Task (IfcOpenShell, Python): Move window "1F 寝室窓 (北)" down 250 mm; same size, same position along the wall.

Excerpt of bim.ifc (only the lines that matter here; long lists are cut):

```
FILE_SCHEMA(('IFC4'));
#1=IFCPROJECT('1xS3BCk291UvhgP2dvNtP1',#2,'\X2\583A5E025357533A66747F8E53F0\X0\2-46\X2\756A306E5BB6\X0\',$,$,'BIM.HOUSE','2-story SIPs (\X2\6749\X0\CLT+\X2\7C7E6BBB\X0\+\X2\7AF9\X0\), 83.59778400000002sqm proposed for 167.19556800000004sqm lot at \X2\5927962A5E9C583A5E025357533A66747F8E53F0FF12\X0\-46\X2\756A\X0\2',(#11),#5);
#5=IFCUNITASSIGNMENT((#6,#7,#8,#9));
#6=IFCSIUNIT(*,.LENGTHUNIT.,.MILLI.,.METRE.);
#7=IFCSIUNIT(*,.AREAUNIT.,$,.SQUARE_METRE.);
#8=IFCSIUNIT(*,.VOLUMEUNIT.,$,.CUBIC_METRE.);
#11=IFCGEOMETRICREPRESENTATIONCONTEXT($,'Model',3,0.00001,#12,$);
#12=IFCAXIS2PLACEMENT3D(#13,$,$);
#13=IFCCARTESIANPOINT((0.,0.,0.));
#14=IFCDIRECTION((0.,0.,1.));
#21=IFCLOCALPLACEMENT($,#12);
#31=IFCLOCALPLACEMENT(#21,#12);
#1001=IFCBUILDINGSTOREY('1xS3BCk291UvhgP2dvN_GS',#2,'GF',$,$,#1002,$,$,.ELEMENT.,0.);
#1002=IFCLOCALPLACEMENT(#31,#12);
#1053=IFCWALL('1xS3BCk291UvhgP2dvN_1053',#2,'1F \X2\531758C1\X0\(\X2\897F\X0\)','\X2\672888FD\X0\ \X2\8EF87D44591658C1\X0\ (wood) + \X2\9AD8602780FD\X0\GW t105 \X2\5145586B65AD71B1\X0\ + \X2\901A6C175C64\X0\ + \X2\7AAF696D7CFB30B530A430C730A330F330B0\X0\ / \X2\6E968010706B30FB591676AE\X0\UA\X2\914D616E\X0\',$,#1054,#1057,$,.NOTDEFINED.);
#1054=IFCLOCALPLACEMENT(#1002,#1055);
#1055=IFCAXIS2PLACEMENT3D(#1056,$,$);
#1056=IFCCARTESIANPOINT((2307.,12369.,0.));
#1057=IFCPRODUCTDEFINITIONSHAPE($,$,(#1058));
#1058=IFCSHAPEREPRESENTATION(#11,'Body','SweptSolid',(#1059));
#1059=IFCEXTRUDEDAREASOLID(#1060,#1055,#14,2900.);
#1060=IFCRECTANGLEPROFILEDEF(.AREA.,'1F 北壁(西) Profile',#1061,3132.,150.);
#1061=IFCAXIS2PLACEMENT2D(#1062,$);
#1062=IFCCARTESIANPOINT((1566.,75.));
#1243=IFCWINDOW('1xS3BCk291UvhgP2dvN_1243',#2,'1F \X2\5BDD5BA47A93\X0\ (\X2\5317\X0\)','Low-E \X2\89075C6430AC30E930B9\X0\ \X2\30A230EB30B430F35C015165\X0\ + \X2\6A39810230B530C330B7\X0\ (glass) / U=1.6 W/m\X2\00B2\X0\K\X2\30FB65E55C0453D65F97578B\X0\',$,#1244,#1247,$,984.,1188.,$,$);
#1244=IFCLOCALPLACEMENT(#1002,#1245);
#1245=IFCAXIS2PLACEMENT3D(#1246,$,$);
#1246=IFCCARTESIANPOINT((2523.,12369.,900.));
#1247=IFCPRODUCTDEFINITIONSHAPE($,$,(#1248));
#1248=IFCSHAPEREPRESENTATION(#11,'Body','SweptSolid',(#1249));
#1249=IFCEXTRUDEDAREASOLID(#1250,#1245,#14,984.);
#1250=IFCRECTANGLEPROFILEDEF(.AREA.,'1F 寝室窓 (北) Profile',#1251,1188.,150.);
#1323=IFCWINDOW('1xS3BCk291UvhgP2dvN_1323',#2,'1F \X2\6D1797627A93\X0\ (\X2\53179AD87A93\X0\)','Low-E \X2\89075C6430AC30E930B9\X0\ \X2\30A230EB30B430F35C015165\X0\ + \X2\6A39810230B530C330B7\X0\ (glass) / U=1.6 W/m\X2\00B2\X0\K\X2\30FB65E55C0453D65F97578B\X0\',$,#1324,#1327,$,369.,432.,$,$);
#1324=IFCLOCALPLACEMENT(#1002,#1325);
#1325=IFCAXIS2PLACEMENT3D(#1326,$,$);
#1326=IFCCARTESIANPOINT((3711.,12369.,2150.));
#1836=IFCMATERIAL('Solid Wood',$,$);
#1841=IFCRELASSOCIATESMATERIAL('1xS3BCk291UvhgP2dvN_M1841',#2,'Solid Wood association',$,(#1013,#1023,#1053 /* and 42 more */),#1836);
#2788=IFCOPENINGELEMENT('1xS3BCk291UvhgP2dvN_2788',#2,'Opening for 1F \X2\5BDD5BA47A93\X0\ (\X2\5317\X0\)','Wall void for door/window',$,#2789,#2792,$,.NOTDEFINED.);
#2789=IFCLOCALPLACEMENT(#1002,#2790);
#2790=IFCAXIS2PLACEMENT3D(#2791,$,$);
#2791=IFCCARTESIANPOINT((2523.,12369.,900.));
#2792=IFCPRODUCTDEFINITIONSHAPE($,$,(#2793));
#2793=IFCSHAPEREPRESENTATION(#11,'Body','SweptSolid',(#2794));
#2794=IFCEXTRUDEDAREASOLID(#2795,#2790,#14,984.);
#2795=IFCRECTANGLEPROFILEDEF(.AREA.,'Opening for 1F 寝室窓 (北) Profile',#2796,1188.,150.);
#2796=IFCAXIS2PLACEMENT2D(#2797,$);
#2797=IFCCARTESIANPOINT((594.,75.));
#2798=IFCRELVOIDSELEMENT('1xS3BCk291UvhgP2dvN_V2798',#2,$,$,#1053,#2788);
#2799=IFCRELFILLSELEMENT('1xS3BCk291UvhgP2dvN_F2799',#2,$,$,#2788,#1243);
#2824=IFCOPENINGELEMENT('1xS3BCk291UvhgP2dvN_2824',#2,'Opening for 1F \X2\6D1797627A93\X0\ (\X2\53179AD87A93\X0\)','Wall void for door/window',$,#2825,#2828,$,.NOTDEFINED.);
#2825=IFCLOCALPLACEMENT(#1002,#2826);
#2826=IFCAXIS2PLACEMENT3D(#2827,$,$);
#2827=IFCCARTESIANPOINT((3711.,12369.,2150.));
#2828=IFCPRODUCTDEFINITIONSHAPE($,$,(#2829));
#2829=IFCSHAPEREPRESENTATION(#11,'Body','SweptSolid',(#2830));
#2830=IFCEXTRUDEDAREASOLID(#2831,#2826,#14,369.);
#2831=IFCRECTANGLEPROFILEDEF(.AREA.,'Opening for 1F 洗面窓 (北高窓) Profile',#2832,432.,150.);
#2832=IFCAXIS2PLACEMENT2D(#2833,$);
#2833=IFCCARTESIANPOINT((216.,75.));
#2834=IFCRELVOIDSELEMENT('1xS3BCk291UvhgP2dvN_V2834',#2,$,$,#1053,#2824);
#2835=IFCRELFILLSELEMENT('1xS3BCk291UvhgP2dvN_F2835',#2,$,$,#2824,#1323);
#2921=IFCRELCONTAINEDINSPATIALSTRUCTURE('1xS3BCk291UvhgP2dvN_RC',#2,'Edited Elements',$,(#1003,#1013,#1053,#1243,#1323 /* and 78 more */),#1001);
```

```python
import numpy as np
import ifcopenshell
import ifcopenshell.api.geometry
import ifcopenshell.util.placement
import ifcopenshell.util.unit

model = ifcopenshell.open("bim.ifc")
unit_scale = ifcopenshell.util.unit.calculate_unit_scale(model)

window = model.by_guid("1xS3BCk291UvhgP2dvN_1243")
opening = window.FillsVoids[0].RelatingOpeningElement
dz = -0.25 / unit_scale

shift = np.array([0.0, 0.0, dz])
# The window is not placed relative to its opening, so move both.
for product in (opening, window):
    matrix = ifcopenshell.util.placement.get_local_placement(product.ObjectPlacement)
    matrix[:3, 3] += shift
    ifcopenshell.api.geometry.edit_object_placement(model, product=product, matrix=matrix, is_si=False)

print(f"moved by {dz * unit_scale:+.3f} m")

model.write("bim_edited.ifc")
```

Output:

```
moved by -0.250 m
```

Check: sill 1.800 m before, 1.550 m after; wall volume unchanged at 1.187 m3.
